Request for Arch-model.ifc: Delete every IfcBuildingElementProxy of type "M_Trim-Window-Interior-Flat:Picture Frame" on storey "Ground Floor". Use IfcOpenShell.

First a look at what the model holds.

```python
import ifcopenshell
import ifcopenshell.util.element

model = ifcopenshell.open("Arch-model.ifc")
print(model.schema)
storey = next(s for s in model.by_type("IfcBuildingStorey") if s.Name == "Ground Floor")
proxies = [e for e in ifcopenshell.util.element.get_decomposition(storey) if e.is_a("IfcBuildingElementProxy")]
seen = {}
for e in proxies:
    element_type = ifcopenshell.util.element.get_type(e)
    name = element_type.Name if element_type not in (None, e) else None
    seen[name] = seen.get(name, 0) + 1
for name, count in sorted(seen.items(), key=str):
    print(count, "x", name)
```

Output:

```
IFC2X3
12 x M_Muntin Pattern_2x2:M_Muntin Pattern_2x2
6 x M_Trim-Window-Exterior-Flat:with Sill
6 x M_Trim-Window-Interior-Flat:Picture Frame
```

```python
import ifcopenshell
import ifcopenshell.api.root
import ifcopenshell.util.element

model = ifcopenshell.open("Arch-model.ifc")

storey = next(s for s in model.by_type("IfcBuildingStorey") if s.Name == "Ground Floor")
proxies = [e for e in ifcopenshell.util.element.get_decomposition(storey) if e.is_a("IfcBuildingElementProxy")]
targets = [e for e in proxies if (t := ifcopenshell.util.element.get_type(e)) not in (None, e) and t.Name == "M_Trim-Window-Interior-Flat:Picture Frame"]

for e in targets:
    ifcopenshell.api.root.remove_product(model, product=e)
print(len(targets), "removed")

model.write("Arch-model_rev.ifc")
```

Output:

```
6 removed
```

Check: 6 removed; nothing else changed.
